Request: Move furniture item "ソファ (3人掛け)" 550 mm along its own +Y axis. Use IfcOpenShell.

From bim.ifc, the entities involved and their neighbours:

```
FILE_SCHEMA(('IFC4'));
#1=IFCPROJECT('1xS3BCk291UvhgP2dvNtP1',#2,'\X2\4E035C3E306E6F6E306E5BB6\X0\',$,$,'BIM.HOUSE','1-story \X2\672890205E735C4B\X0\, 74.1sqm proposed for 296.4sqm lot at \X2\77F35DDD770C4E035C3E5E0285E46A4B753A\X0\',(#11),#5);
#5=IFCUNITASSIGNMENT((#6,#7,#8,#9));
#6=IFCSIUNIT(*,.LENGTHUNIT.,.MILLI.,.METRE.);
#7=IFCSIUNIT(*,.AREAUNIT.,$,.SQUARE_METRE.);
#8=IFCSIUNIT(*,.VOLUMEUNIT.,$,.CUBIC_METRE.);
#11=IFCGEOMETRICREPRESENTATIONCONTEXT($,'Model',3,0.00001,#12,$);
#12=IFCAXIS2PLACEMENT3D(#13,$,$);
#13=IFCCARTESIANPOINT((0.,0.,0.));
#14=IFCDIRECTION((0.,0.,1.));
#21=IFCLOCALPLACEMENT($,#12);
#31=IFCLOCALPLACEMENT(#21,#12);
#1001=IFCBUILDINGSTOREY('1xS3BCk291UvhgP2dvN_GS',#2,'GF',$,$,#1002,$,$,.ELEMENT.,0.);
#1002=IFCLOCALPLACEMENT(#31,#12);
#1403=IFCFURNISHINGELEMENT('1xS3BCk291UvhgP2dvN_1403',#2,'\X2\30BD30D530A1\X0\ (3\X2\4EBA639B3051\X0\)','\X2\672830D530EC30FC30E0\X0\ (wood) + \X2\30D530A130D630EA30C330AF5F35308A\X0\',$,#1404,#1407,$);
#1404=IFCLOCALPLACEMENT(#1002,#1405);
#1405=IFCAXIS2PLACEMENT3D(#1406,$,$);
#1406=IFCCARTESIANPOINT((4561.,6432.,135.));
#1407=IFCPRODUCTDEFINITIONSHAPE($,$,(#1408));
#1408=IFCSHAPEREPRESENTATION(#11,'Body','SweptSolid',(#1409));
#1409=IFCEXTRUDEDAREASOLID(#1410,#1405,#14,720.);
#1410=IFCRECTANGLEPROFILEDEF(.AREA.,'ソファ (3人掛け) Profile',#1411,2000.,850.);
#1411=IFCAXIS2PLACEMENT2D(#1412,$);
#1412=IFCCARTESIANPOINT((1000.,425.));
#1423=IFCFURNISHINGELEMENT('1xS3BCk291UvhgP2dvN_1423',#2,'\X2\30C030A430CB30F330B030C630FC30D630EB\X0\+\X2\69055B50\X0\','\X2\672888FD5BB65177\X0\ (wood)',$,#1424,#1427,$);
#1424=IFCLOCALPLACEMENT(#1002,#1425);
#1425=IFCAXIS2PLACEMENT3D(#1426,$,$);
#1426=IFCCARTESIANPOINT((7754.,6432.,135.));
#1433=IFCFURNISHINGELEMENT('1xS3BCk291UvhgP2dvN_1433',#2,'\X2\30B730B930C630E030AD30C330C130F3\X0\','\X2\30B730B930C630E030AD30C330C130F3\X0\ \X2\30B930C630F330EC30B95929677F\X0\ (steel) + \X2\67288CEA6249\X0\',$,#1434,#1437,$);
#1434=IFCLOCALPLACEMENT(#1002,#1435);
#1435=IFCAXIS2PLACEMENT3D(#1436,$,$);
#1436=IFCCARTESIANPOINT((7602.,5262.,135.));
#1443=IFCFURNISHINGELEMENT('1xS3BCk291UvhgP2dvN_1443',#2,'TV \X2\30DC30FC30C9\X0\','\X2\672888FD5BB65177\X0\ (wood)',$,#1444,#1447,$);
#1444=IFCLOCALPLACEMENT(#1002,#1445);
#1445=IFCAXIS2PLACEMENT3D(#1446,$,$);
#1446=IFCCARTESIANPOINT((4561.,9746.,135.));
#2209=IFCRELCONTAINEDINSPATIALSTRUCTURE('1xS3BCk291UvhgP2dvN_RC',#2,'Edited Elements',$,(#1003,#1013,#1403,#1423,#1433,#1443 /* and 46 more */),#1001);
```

```python
import ifcopenshell
import ifcopenshell.api.geometry
import ifcopenshell.util.placement
import ifcopenshell.util.unit

model = ifcopenshell.open("bim.ifc")
unit_scale = ifcopenshell.util.unit.calculate_unit_scale(model)

item = model.by_guid("1xS3BCk291UvhgP2dvN_1403")
matrix = ifcopenshell.util.placement.get_local_placement(item.ObjectPlacement)
matrix[:3, 3] += matrix[:3, 1] * 0.55 / unit_scale
ifcopenshell.api.geometry.edit_object_placement(model, product=item, matrix=matrix, is_si=False)

print(ifcopenshell.util.placement.get_local_placement(item.ObjectPlacement).round(3) + 0.0)

model.write("bim_updated.ifc")
```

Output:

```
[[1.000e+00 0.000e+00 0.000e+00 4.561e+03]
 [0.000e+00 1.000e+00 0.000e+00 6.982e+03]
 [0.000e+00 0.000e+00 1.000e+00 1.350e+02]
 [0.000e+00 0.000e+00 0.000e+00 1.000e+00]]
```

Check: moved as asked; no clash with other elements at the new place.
